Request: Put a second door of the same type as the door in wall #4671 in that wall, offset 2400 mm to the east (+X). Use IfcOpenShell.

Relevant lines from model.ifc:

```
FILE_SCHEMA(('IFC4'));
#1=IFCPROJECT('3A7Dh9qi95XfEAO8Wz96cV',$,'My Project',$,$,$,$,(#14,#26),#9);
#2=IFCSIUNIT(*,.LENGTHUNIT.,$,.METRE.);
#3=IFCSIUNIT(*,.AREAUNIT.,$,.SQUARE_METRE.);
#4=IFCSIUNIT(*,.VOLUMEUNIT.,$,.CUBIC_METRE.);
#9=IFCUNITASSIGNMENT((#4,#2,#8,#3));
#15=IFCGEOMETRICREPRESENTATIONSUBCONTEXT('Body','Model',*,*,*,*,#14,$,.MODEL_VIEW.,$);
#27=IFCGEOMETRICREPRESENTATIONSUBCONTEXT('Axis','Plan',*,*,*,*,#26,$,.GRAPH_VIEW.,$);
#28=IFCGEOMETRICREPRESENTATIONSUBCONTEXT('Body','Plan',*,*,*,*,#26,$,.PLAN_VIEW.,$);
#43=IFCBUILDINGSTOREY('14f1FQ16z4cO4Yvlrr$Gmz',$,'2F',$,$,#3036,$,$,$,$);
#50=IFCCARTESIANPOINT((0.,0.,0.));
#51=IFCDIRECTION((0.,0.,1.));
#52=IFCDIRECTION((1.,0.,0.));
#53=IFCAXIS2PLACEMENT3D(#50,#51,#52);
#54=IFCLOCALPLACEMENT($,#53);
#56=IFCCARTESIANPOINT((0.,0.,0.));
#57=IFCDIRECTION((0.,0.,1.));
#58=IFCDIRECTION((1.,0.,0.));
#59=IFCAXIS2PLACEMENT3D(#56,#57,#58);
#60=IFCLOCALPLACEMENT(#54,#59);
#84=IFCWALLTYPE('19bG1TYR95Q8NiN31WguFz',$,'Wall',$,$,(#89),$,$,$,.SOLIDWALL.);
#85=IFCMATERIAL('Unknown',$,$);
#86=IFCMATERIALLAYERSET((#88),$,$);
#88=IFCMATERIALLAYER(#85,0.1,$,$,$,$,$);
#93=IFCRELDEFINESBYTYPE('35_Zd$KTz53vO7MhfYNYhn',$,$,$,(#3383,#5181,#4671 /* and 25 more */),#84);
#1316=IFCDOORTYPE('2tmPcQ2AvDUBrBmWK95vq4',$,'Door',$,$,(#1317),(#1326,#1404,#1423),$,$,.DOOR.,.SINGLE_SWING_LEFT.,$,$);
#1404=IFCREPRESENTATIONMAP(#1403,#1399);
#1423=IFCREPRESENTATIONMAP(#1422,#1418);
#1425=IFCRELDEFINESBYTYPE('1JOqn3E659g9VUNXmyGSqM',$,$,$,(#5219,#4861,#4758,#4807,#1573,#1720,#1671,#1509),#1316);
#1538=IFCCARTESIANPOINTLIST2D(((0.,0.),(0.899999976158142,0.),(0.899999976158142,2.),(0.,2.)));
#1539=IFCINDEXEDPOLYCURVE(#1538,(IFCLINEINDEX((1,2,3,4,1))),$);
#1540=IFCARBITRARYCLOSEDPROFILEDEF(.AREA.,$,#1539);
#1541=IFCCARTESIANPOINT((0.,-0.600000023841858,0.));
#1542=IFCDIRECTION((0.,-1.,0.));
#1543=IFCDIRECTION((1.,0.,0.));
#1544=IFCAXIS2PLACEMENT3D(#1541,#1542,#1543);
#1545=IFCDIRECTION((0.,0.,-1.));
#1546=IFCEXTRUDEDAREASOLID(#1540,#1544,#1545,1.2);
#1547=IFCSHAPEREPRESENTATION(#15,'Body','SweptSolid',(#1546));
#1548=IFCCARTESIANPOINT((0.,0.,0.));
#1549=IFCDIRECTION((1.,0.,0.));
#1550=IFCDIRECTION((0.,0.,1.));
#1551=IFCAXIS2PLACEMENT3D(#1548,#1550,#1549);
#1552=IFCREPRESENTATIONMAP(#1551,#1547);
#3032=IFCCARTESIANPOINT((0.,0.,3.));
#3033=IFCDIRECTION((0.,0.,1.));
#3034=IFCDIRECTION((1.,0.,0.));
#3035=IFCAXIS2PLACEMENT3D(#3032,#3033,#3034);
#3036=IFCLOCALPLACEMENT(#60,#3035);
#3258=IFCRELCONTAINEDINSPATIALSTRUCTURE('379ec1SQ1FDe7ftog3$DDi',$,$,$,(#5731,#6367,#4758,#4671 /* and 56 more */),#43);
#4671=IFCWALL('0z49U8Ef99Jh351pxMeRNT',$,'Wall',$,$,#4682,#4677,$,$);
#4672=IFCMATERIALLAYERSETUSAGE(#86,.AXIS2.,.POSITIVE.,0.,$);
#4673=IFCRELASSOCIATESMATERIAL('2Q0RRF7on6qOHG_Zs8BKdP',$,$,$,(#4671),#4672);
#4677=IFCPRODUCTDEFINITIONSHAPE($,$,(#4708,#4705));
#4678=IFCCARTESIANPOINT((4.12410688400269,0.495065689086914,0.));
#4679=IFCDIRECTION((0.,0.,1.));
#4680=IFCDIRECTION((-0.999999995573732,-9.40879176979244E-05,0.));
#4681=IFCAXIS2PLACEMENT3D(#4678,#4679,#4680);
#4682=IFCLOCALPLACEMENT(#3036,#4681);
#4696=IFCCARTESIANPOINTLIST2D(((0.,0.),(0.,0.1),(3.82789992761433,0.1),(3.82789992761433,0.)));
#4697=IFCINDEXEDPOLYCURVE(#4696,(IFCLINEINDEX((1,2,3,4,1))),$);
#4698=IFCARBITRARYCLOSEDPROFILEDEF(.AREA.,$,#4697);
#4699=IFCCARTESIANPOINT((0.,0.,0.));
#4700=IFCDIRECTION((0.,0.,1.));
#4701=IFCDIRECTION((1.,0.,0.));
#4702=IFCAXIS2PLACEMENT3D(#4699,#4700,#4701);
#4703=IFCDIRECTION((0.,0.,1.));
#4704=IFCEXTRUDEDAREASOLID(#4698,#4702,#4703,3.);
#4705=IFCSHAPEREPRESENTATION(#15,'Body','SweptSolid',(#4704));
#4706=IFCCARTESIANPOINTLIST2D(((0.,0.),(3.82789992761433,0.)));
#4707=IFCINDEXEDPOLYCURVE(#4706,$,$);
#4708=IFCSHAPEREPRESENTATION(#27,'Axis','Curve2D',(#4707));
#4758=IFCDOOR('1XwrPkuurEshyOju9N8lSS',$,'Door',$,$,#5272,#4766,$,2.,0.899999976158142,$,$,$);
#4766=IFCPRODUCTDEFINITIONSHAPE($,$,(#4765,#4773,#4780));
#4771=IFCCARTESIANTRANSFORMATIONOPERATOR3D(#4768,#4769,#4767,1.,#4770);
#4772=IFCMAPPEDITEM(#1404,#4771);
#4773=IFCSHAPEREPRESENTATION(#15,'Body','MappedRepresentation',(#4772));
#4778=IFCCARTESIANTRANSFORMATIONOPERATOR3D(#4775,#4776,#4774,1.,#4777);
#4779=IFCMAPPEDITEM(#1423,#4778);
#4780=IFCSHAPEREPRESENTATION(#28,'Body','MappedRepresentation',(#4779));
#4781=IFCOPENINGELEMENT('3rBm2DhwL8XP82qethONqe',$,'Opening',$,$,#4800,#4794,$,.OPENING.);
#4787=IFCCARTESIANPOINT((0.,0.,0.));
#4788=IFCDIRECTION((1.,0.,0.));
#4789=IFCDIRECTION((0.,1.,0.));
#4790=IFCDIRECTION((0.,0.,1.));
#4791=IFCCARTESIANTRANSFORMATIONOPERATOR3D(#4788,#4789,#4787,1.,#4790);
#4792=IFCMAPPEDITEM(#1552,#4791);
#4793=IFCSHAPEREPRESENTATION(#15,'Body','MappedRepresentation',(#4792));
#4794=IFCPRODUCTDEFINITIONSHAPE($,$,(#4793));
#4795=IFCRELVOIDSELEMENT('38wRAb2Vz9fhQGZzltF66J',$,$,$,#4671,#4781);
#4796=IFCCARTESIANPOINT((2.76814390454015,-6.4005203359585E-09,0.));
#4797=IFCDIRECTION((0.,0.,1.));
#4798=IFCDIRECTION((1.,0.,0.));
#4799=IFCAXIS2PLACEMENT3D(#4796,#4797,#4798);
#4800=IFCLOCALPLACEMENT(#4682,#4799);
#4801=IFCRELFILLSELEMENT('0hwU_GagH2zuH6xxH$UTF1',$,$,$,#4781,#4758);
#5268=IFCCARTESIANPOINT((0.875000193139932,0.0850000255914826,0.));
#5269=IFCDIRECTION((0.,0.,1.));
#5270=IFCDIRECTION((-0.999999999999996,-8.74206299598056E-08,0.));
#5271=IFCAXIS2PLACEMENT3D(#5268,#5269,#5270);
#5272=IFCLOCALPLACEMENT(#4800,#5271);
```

```python
import ifcopenshell
import ifcopenshell.api.feature
import ifcopenshell.api.geometry
import ifcopenshell.api.root
import ifcopenshell.geom
import ifcopenshell.util.element
import ifcopenshell.util.placement
import ifcopenshell.util.shape
import ifcopenshell.util.unit

model = ifcopenshell.open("model.ifc")
unit_scale = ifcopenshell.util.unit.calculate_unit_scale(model)
settings = ifcopenshell.geom.settings()


def volume(element):
    """Net volume in cubic metres, openings subtracted."""
    shape = ifcopenshell.geom.create_shape(settings, element)
    return ifcopenshell.util.shape.get_volume(shape.geometry)


door = model.by_guid("1XwrPkuurEshyOju9N8lSS")
opening = door.FillsVoids[0].RelatingOpeningElement
wall = opening.VoidsElements[0].RelatingBuildingElement
before = volume(wall)
shift = ifcopenshell.util.placement.get_local_placement(wall.ObjectPlacement)[:3, 0] * -2.4 / unit_scale

# copy_class copies the void relationship, type, container and properties, but no geometry.
new_opening = ifcopenshell.api.root.copy_class(model, product=opening)
new_opening.Representation = ifcopenshell.util.element.copy_deep(
    model, opening.Representation, exclude=["IfcGeometricRepresentationContext", "IfcRepresentationMap"]
)
new_door = ifcopenshell.api.root.copy_class(model, product=door)
new_door.Representation = ifcopenshell.util.element.copy_deep(
    model, door.Representation, exclude=["IfcGeometricRepresentationContext", "IfcRepresentationMap"]
)
ifcopenshell.api.feature.add_filling(model, opening=new_opening, element=new_door)

for old, new in ((opening, new_opening), (door, new_door)):
    matrix = ifcopenshell.util.placement.get_local_placement(old.ObjectPlacement)
    matrix[:3, 3] += shift
    ifcopenshell.api.geometry.edit_object_placement(model, product=new, matrix=matrix, is_si=False)

after = volume(wall)

print(f"wall volume {before:.3f} -> {after:.3f} m3")

model.write("model_rev.ifc")
```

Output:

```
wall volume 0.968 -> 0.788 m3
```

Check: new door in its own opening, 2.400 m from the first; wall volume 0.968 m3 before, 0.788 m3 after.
